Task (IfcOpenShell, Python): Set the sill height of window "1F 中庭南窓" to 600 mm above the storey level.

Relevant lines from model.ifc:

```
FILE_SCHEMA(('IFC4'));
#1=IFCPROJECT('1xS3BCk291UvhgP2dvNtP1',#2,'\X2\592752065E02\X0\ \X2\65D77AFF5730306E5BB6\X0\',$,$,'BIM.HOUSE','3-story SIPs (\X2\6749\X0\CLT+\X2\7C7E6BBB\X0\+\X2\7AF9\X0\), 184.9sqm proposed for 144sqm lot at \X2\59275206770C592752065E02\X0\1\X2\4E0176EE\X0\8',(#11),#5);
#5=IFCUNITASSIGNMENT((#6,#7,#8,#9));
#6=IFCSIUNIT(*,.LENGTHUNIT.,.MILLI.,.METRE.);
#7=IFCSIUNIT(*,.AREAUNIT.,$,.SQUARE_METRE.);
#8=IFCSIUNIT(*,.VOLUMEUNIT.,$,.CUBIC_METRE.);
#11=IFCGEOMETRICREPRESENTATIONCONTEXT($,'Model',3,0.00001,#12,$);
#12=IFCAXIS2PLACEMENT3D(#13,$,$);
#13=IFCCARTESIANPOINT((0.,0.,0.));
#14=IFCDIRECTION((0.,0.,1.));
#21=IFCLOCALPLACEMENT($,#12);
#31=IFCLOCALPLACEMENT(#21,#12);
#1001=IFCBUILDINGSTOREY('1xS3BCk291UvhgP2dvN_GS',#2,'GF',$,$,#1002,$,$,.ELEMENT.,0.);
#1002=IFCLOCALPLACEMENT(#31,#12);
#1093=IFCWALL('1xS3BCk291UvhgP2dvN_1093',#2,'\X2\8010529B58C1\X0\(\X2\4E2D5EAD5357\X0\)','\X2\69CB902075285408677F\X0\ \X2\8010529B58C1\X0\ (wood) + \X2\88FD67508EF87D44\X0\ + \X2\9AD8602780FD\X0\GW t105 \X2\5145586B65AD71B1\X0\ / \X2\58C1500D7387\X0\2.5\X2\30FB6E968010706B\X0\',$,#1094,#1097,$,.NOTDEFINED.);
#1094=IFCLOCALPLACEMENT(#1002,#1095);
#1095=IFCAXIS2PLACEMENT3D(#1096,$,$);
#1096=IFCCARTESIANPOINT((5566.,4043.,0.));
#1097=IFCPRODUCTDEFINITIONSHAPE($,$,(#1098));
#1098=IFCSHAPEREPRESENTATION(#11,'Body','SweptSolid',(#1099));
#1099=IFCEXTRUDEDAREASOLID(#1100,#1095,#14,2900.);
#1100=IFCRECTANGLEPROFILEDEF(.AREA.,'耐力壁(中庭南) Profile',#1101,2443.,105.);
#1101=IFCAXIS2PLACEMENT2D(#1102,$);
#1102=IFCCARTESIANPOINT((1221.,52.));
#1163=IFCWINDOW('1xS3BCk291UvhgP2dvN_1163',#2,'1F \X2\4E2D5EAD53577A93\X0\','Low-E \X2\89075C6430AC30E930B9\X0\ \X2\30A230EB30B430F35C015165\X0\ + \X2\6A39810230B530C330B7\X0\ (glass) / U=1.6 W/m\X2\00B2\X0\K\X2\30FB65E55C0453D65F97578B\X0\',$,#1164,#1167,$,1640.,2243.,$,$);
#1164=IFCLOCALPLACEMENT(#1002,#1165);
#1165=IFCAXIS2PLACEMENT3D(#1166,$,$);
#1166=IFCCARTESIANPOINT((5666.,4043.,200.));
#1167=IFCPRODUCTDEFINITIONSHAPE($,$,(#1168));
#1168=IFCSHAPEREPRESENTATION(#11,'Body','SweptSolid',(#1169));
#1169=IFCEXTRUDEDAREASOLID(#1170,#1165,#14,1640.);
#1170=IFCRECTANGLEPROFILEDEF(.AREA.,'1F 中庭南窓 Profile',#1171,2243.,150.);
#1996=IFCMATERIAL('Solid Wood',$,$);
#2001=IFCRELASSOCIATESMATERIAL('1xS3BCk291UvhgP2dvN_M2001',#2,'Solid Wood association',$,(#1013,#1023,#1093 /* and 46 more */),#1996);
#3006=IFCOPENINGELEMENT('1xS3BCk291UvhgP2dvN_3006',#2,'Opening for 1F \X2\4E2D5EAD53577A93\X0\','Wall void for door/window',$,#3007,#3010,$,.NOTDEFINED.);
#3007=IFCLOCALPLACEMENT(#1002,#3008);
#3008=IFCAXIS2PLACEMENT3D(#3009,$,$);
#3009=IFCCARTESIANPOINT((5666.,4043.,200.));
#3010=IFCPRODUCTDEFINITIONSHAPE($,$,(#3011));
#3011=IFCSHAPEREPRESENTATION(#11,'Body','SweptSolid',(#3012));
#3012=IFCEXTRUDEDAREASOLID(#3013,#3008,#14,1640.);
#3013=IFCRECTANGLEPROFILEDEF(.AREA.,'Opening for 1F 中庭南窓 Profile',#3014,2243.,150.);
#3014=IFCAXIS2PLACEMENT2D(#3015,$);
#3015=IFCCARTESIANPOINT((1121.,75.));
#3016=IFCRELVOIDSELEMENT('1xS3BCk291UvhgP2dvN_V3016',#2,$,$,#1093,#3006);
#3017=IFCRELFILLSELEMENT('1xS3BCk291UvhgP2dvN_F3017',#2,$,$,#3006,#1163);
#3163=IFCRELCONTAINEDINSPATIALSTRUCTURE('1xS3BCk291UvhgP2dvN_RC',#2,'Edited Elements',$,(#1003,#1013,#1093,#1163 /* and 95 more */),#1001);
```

```python
import numpy as np
import ifcopenshell
import ifcopenshell.api.geometry
import ifcopenshell.geom
import ifcopenshell.util.element
import ifcopenshell.util.placement
import ifcopenshell.util.shape
import ifcopenshell.util.unit

model = ifcopenshell.open("model.ifc")
unit_scale = ifcopenshell.util.unit.calculate_unit_scale(model)

window = model.by_guid("1xS3BCk291UvhgP2dvN_1163")
opening = window.FillsVoids[0].RelatingOpeningElement
storey = ifcopenshell.util.element.get_container(window, ifc_class="IfcBuildingStorey")
level = ifcopenshell.util.placement.get_local_placement(storey.ObjectPlacement)[2, 3]

# The opening's origin need not be at the sill, so measure its lowest point.
shape = ifcopenshell.geom.create_shape(ifcopenshell.geom.settings(), opening)
bottom = ifcopenshell.util.shape.get_shape_bottom_elevation(shape, shape.geometry) / unit_scale
dz = level + 0.6 / unit_scale - bottom

shift = np.array([0.0, 0.0, dz])
# The window is not placed relative to its opening, so move both.
for product in (opening, window):
    matrix = ifcopenshell.util.placement.get_local_placement(product.ObjectPlacement)
    matrix[:3, 3] += shift
    ifcopenshell.api.geometry.edit_object_placement(model, product=product, matrix=matrix, is_si=False)

print(f"moved by {dz * unit_scale:+.3f} m")

model.write("model_rev.ifc")
```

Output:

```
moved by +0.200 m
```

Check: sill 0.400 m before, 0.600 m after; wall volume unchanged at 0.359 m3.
